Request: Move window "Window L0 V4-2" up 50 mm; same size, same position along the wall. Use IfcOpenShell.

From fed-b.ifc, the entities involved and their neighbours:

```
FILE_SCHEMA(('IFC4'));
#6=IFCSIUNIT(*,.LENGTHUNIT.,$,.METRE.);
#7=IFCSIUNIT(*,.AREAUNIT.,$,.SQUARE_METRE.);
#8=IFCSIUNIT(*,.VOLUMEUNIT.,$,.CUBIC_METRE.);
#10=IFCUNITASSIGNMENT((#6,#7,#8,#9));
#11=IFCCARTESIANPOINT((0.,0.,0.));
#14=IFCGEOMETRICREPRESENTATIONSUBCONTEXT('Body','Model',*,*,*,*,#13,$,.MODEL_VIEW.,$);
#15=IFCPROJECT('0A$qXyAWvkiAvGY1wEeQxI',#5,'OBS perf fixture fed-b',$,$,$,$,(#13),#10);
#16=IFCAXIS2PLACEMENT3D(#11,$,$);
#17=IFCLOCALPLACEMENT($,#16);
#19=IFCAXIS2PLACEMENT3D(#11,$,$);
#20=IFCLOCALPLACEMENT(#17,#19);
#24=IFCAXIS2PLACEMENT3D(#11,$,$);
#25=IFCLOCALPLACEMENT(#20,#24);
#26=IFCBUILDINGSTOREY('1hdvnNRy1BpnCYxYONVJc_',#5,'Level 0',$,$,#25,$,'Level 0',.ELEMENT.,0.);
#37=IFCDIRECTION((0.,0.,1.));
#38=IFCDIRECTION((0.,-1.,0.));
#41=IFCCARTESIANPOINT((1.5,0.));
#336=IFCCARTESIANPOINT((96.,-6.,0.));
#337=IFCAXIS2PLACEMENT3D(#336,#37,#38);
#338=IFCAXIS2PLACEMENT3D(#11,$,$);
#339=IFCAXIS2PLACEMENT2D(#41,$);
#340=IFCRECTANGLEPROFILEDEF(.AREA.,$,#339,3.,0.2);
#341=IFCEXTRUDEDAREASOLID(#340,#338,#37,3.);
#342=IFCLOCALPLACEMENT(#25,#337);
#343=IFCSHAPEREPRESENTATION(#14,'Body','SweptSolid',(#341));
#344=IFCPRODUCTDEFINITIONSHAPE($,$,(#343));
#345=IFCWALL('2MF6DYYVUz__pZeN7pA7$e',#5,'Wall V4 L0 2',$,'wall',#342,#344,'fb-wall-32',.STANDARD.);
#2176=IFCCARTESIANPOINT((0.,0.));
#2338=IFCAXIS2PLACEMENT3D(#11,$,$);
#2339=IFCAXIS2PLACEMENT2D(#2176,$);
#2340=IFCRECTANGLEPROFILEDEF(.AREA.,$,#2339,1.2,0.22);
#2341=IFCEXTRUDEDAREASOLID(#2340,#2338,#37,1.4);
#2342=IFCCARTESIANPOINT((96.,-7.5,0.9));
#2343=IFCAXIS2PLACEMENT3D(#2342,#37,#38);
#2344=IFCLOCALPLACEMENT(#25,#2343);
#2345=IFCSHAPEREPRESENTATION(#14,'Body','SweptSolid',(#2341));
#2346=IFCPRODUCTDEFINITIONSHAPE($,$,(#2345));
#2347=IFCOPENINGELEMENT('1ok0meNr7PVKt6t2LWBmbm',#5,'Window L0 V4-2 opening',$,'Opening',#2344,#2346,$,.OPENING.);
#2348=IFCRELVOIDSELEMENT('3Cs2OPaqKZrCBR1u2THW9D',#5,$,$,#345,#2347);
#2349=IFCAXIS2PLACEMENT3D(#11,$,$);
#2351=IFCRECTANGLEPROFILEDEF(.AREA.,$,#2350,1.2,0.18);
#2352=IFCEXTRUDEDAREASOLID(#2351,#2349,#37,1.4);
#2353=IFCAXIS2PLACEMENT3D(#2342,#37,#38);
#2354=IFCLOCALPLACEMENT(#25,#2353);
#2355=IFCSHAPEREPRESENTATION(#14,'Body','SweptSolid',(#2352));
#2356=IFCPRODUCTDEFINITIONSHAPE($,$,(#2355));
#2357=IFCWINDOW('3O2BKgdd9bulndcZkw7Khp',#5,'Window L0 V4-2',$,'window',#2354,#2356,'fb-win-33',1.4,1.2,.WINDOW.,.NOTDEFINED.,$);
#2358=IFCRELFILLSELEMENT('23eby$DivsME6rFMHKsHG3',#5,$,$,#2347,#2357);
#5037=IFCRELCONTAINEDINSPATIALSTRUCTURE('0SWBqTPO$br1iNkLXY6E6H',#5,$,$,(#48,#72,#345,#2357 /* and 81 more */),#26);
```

```python
import numpy as np
import ifcopenshell
import ifcopenshell.api.geometry
import ifcopenshell.util.placement
import ifcopenshell.util.unit

model = ifcopenshell.open("fed-b.ifc")
unit_scale = ifcopenshell.util.unit.calculate_unit_scale(model)

window = model.by_id(2357)
opening = window.FillsVoids[0].RelatingOpeningElement
dz = 0.05

shift = np.array([0.0, 0.0, dz])
# The window is not placed relative to its opening, so move both.
for product in (opening, window):
    matrix = ifcopenshell.util.placement.get_local_placement(product.ObjectPlacement)
    matrix[:3, 3] += shift
    ifcopenshell.api.geometry.edit_object_placement(model, product=product, matrix=matrix, is_si=False)

print(f"moved by {dz * unit_scale:+.3f} m")

model.write("fed-b_updated.ifc")
```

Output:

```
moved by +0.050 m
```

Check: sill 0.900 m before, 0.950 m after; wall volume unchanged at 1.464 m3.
